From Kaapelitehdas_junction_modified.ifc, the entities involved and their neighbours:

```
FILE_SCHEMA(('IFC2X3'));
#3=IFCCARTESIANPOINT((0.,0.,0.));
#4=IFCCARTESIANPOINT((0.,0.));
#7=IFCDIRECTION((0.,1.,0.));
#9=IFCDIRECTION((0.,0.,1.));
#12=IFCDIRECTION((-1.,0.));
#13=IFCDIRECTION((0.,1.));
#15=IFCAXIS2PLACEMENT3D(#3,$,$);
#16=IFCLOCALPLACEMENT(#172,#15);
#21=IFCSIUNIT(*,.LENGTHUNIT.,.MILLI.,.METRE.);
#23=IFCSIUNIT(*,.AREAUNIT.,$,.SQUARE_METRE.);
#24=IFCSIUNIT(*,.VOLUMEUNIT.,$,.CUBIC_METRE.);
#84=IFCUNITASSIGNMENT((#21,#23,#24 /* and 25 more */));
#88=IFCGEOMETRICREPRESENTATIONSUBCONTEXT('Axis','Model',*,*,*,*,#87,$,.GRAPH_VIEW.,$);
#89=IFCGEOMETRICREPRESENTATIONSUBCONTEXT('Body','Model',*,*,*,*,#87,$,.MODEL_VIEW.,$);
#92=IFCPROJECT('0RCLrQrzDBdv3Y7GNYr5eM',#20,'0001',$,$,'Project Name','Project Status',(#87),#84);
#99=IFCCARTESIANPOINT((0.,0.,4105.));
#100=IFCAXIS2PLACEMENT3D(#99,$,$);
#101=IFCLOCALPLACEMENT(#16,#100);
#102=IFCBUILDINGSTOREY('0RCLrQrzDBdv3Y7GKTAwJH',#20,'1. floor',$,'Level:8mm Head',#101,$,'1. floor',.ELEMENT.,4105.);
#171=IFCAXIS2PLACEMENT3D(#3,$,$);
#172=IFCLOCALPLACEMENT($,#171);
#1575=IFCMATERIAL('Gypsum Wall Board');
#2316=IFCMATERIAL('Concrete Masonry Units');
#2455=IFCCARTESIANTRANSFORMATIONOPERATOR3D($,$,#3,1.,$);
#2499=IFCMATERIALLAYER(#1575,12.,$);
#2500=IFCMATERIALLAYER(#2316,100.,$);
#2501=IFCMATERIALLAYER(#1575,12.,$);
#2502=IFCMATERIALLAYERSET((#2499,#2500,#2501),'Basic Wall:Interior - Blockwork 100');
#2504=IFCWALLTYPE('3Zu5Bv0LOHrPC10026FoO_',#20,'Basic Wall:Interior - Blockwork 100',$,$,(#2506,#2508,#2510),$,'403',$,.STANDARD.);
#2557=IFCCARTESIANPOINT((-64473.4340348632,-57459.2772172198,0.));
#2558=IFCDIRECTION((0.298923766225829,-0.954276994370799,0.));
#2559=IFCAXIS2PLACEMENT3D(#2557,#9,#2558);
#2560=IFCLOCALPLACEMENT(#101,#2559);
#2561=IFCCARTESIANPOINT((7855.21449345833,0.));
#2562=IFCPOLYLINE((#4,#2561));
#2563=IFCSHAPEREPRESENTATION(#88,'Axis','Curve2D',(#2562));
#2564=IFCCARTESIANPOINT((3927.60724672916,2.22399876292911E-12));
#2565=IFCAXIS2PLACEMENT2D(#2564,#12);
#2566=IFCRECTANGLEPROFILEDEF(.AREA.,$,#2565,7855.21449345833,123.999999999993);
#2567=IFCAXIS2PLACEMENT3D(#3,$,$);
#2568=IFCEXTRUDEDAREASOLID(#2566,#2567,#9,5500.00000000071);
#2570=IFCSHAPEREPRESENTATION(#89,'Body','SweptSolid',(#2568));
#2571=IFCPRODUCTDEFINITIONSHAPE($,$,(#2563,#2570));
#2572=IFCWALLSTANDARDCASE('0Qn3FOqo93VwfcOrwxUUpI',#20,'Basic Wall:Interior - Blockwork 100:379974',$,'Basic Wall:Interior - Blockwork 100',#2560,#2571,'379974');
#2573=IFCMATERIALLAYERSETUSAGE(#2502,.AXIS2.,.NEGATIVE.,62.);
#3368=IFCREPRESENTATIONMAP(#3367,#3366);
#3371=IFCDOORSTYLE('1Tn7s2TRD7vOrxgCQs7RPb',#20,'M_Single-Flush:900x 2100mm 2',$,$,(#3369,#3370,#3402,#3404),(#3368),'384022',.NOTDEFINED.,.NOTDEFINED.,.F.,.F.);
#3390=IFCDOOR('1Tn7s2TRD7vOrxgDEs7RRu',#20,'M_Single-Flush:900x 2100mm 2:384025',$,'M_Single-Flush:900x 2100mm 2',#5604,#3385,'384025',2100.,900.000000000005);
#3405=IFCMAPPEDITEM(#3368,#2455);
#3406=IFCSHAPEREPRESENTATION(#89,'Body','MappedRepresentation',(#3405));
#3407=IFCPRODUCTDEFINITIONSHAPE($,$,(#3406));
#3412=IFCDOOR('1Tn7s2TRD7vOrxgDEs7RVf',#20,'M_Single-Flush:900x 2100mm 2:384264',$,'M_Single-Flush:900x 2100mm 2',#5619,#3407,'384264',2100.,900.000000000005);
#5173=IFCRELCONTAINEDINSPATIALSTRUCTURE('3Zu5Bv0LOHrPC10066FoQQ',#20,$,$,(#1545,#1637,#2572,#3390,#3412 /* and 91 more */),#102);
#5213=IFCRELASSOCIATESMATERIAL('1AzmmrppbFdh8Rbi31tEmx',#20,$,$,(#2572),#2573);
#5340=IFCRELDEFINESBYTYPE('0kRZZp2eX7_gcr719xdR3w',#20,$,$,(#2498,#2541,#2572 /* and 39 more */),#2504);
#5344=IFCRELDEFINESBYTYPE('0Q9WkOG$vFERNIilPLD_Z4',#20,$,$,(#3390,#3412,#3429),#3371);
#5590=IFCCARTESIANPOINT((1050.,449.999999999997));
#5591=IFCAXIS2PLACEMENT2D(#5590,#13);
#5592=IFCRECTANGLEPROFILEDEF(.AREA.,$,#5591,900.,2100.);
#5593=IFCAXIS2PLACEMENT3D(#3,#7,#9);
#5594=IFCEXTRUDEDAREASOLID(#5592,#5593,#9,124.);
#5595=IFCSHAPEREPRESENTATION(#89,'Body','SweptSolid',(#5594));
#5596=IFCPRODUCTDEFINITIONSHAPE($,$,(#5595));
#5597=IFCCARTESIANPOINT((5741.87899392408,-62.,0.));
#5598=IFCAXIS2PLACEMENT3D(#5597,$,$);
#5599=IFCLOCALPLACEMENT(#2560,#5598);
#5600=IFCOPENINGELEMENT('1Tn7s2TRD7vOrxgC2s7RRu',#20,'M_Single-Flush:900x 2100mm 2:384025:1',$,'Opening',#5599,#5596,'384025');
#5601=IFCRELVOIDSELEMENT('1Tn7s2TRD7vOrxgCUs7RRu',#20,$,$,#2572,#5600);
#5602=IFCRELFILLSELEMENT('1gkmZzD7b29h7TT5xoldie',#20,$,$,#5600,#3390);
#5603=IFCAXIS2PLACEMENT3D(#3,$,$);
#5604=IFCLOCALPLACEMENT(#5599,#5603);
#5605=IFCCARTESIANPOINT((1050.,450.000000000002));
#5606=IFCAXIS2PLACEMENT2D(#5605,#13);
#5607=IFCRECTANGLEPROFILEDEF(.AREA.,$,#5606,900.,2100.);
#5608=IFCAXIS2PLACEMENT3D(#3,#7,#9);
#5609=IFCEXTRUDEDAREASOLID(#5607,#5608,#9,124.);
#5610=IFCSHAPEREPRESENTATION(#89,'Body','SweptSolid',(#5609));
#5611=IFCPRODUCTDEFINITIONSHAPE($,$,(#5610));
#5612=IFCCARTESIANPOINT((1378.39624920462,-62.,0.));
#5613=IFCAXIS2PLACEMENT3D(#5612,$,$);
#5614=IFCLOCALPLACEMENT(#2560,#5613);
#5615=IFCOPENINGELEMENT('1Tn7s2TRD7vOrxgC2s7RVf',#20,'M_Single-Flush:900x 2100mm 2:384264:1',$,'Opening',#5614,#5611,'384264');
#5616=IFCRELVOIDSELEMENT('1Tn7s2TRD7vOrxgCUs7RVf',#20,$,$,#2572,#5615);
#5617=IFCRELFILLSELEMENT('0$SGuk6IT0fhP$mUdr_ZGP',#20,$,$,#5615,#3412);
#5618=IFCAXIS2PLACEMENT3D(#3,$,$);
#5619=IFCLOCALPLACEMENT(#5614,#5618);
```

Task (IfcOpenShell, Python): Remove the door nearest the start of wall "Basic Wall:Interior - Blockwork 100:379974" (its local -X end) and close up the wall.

```python
import ifcopenshell
import ifcopenshell.api.feature
import ifcopenshell.api.root
import ifcopenshell.geom
import ifcopenshell.util.shape

model = ifcopenshell.open("Kaapelitehdas_junction_modified.ifc")
settings = ifcopenshell.geom.settings()


def volume(element):
    """Net volume in cubic metres, openings subtracted."""
    shape = ifcopenshell.geom.create_shape(settings, element)
    return ifcopenshell.util.shape.get_volume(shape.geometry)


door = model.by_guid("1Tn7s2TRD7vOrxgDEs7RVf")
opening = door.FillsVoids[0].RelatingOpeningElement
wall = opening.VoidsElements[0].RelatingBuildingElement
before = volume(wall)

ifcopenshell.api.root.remove_product(model, product=door)
ifcopenshell.api.feature.remove_feature(model, feature=opening)

after = volume(wall)

print(f"wall volume {before:.3f} -> {after:.3f} m3")

model.write("Kaapelitehdas_junction_modified_rev.ifc")
```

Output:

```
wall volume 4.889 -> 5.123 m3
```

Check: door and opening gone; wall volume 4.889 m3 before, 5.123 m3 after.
